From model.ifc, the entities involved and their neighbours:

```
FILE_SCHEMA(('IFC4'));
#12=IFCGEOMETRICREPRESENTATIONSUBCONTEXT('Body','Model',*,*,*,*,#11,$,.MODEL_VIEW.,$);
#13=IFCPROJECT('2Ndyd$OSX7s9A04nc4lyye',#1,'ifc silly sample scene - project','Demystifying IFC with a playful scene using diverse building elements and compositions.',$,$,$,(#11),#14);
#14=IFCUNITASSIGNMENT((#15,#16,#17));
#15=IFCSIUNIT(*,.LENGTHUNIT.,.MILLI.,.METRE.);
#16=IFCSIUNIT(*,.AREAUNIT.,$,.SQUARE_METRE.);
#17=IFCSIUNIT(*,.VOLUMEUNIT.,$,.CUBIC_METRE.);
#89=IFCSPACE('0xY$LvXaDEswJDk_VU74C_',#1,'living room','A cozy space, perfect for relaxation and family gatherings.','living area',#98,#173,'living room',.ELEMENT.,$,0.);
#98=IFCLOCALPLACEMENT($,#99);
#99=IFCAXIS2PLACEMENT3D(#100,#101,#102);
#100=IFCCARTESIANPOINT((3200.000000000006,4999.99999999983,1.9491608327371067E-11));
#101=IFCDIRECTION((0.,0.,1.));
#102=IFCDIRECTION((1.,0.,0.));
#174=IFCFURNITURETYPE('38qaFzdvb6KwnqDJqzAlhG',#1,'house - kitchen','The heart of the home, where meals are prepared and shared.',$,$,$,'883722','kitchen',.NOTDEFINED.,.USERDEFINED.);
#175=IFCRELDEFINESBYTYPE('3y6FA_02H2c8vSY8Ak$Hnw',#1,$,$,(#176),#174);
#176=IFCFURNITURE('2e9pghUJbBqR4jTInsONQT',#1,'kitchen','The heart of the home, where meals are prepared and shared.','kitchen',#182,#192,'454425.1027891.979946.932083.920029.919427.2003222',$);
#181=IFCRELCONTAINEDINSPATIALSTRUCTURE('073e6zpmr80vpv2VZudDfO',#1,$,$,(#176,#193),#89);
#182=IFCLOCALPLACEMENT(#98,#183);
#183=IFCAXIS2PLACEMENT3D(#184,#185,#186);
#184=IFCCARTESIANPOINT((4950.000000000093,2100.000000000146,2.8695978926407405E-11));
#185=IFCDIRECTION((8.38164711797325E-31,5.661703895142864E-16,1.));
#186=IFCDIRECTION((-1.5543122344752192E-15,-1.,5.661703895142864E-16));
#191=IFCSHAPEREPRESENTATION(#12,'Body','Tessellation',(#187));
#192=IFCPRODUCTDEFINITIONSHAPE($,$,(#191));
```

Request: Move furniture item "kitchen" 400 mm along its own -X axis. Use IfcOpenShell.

```python
import ifcopenshell
import ifcopenshell.api.geometry
import ifcopenshell.util.placement

model = ifcopenshell.open("model.ifc")

item = model.by_guid("2e9pghUJbBqR4jTInsONQT")
matrix = ifcopenshell.util.placement.get_local_placement(item.ObjectPlacement)
matrix[:3, 3] -= matrix[:3, 0] * 400.0
ifcopenshell.api.geometry.edit_object_placement(model, product=item, matrix=matrix, is_si=False)

print(ifcopenshell.util.placement.get_local_placement(item.ObjectPlacement).round(3) + 0.0)

model.write("model_edited.ifc")
```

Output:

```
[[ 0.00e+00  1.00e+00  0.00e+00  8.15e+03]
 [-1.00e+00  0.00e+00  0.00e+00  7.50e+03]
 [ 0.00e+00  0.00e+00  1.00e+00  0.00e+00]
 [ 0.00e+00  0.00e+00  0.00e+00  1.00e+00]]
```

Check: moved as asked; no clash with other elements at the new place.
